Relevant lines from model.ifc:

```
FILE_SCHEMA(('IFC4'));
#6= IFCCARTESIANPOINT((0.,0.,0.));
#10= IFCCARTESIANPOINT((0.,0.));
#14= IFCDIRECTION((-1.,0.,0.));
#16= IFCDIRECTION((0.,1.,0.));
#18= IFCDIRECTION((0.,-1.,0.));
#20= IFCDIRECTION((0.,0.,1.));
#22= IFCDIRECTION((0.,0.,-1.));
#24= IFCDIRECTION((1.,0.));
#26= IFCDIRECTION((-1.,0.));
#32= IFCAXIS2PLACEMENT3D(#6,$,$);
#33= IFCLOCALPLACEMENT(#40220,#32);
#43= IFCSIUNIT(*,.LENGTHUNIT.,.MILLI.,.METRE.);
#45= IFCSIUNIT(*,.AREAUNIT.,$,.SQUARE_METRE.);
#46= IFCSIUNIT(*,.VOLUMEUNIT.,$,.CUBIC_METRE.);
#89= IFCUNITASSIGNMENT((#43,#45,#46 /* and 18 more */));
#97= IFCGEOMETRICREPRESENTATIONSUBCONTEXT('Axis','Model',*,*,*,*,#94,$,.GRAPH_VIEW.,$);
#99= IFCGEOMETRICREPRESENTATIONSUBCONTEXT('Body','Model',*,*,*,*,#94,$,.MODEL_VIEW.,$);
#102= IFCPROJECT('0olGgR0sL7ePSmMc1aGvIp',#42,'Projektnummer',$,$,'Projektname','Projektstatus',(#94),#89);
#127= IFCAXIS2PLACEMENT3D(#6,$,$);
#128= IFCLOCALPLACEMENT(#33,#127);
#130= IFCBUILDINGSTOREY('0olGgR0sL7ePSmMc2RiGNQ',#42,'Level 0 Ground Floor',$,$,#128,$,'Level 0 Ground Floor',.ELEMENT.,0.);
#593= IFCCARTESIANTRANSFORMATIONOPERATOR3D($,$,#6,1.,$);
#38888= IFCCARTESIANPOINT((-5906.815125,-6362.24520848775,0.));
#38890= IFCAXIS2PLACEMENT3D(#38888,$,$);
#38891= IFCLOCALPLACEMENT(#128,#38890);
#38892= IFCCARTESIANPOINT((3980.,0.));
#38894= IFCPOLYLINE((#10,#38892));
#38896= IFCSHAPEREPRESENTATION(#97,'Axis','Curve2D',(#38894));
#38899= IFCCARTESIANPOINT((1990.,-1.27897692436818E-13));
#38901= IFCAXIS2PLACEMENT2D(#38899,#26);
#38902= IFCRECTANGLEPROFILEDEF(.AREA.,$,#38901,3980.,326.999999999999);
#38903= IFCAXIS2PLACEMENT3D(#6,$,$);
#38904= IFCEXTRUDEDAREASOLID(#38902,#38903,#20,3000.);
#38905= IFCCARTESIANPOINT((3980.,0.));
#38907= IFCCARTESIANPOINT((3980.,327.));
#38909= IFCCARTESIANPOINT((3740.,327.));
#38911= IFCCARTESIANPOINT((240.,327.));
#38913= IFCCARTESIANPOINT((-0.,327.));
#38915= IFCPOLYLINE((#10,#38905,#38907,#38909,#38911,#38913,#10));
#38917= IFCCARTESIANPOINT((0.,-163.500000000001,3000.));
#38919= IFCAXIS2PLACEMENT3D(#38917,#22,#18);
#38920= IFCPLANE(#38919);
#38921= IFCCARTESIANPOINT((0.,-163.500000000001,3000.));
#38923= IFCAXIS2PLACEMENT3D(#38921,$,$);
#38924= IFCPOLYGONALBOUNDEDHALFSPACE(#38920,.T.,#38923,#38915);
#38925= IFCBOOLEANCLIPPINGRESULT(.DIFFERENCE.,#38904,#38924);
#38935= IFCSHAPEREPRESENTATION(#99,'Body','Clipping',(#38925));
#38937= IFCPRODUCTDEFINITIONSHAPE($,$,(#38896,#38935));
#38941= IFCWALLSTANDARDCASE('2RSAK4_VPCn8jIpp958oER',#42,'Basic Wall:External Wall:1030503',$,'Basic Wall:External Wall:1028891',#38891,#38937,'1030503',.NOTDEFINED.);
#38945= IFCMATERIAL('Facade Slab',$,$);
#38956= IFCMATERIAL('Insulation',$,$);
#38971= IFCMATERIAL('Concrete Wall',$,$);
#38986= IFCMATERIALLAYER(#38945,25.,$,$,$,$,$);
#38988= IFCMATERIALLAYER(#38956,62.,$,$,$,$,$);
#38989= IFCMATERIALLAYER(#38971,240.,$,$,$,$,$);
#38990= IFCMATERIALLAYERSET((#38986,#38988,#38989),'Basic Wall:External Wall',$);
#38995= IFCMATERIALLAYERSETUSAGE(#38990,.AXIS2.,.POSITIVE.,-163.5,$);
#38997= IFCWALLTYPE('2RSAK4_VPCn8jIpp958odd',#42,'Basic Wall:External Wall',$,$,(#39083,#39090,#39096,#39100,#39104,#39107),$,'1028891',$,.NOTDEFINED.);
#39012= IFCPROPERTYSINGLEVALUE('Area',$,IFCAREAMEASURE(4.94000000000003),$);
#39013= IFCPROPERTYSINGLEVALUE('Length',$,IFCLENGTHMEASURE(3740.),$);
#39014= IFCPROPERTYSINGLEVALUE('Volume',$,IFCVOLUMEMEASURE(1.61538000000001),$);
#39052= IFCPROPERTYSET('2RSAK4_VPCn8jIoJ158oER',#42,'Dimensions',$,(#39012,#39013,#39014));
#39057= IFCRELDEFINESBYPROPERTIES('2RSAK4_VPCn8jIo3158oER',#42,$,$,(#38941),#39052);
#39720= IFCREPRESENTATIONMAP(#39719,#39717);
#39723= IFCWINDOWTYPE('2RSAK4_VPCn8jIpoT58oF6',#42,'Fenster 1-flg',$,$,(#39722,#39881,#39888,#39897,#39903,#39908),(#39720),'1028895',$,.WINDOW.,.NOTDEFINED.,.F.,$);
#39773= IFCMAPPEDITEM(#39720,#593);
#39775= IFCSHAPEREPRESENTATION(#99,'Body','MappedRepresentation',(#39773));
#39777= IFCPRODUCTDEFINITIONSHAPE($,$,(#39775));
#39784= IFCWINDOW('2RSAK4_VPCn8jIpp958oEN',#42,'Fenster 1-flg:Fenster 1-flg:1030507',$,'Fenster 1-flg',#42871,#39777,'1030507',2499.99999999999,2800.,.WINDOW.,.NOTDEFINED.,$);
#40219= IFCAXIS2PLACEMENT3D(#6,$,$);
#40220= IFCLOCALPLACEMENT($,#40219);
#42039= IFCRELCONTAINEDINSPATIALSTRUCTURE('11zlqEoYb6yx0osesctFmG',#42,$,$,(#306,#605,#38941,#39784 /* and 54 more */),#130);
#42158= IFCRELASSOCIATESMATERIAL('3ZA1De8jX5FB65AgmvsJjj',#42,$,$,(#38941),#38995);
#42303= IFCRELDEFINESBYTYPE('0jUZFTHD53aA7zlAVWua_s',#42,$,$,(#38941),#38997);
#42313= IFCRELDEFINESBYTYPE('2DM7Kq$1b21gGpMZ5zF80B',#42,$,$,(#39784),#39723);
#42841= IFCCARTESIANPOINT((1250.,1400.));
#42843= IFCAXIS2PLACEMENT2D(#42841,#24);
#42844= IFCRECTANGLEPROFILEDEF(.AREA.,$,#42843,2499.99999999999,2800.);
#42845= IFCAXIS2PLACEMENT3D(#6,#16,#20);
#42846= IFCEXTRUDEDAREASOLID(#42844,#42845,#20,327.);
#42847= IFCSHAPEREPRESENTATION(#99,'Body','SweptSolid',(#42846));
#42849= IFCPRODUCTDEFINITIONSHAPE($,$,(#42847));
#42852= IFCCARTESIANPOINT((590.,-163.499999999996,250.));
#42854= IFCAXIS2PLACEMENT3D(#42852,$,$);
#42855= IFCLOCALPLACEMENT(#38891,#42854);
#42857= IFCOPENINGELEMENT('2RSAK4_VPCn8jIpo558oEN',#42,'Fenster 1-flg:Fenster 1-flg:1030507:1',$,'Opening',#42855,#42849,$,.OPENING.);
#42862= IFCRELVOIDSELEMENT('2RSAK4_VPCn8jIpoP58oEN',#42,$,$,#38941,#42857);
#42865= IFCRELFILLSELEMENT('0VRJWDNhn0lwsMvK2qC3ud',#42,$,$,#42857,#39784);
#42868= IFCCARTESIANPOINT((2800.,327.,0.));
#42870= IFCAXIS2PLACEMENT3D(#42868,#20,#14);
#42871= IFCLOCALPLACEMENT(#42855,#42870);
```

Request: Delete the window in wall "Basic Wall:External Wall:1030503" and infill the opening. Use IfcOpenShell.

```python
import ifcopenshell
import ifcopenshell.api.feature
import ifcopenshell.api.pset
import ifcopenshell.api.root
import ifcopenshell.geom
import ifcopenshell.util.element
import ifcopenshell.util.shape
import ifcopenshell.util.unit

model = ifcopenshell.open("model.ifc")
area_scale = ifcopenshell.util.unit.calculate_unit_scale(model, "AREAUNIT")
volume_scale = ifcopenshell.util.unit.calculate_unit_scale(model, "VOLUMEUNIT")
settings = ifcopenshell.geom.settings()


def volume(element):
    """Net volume in cubic metres, openings subtracted."""
    shape = ifcopenshell.geom.create_shape(settings, element)
    return ifcopenshell.util.shape.get_volume(shape.geometry)


window = model.by_id(39784)
opening = window.FillsVoids[0].RelatingOpeningElement
wall = opening.VoidsElements[0].RelatingBuildingElement
before = volume(wall)

ifcopenshell.api.root.remove_product(model, product=window)
ifcopenshell.api.feature.remove_feature(model, feature=opening)

after = volume(wall)
thickness = 0.327  # wall thickness in metres

# Update the wall's stored quantities.
pset = model.by_id(ifcopenshell.util.element.get_pset(wall, "Dimensions", should_inherit=False)["id"])
ifcopenshell.api.pset.edit_pset(model, pset=pset, properties={
    "Area": model.create_entity("IfcAreaMeasure", after / thickness / area_scale),
    "Volume": model.create_entity("IfcVolumeMeasure", after / volume_scale),
})

print(f"wall volume {before:.3f} -> {after:.3f} m3")

model.write("model_updated.ifc")
```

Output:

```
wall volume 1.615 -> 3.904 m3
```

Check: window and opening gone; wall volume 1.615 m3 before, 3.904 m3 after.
